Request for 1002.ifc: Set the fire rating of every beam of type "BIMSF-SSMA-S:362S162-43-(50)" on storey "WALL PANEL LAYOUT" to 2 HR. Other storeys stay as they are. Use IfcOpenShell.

First a look at what the model holds.

```python
import ifcopenshell
import ifcopenshell.util.element

model = ifcopenshell.open("1002.ifc")
print(model.schema)
storey = next(s for s in model.by_type("IfcBuildingStorey") if s.Name == "WALL PANEL LAYOUT")
beams = [e for e in ifcopenshell.util.element.get_decomposition(storey) if e.is_a("IfcBeam")]
seen = {}
for e in beams:
    element_type = ifcopenshell.util.element.get_type(e)
    key = (element_type.Name if element_type != e and element_type else None, ifcopenshell.util.element.get_pset(e, "Pset_BeamCommon", "FireRating"))
    seen[key] = seen.get(key, 0) + 1
for (name, value), count in sorted(seen.items(), key=str):
    print(count, "x", name, "|", value)
```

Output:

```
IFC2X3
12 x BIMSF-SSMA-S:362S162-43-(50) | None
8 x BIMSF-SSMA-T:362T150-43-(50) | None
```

```python
import ifcopenshell
import ifcopenshell.api.pset
import ifcopenshell.util.element

model = ifcopenshell.open("1002.ifc")

storey = next(s for s in model.by_type("IfcBuildingStorey") if s.Name == "WALL PANEL LAYOUT")
beams = [e for e in ifcopenshell.util.element.get_decomposition(storey) if e.is_a("IfcBeam")]

count = 0
for e in beams:
    element_type = ifcopenshell.util.element.get_type(e)
    if element_type in (None, e) or element_type.Name != "BIMSF-SSMA-S:362S162-43-(50)":
        continue
    # add_pset returns the element's existing set when there is one.
    pset = ifcopenshell.api.pset.add_pset(model, product=e, name="Pset_BeamCommon")
    ifcopenshell.api.pset.edit_pset(model, pset=pset, properties={"FireRating": "2 HR"})
    count += 1

print(count, "beams updated")

model.write("1002_rev.ifc")
```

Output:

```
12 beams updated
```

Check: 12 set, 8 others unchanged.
